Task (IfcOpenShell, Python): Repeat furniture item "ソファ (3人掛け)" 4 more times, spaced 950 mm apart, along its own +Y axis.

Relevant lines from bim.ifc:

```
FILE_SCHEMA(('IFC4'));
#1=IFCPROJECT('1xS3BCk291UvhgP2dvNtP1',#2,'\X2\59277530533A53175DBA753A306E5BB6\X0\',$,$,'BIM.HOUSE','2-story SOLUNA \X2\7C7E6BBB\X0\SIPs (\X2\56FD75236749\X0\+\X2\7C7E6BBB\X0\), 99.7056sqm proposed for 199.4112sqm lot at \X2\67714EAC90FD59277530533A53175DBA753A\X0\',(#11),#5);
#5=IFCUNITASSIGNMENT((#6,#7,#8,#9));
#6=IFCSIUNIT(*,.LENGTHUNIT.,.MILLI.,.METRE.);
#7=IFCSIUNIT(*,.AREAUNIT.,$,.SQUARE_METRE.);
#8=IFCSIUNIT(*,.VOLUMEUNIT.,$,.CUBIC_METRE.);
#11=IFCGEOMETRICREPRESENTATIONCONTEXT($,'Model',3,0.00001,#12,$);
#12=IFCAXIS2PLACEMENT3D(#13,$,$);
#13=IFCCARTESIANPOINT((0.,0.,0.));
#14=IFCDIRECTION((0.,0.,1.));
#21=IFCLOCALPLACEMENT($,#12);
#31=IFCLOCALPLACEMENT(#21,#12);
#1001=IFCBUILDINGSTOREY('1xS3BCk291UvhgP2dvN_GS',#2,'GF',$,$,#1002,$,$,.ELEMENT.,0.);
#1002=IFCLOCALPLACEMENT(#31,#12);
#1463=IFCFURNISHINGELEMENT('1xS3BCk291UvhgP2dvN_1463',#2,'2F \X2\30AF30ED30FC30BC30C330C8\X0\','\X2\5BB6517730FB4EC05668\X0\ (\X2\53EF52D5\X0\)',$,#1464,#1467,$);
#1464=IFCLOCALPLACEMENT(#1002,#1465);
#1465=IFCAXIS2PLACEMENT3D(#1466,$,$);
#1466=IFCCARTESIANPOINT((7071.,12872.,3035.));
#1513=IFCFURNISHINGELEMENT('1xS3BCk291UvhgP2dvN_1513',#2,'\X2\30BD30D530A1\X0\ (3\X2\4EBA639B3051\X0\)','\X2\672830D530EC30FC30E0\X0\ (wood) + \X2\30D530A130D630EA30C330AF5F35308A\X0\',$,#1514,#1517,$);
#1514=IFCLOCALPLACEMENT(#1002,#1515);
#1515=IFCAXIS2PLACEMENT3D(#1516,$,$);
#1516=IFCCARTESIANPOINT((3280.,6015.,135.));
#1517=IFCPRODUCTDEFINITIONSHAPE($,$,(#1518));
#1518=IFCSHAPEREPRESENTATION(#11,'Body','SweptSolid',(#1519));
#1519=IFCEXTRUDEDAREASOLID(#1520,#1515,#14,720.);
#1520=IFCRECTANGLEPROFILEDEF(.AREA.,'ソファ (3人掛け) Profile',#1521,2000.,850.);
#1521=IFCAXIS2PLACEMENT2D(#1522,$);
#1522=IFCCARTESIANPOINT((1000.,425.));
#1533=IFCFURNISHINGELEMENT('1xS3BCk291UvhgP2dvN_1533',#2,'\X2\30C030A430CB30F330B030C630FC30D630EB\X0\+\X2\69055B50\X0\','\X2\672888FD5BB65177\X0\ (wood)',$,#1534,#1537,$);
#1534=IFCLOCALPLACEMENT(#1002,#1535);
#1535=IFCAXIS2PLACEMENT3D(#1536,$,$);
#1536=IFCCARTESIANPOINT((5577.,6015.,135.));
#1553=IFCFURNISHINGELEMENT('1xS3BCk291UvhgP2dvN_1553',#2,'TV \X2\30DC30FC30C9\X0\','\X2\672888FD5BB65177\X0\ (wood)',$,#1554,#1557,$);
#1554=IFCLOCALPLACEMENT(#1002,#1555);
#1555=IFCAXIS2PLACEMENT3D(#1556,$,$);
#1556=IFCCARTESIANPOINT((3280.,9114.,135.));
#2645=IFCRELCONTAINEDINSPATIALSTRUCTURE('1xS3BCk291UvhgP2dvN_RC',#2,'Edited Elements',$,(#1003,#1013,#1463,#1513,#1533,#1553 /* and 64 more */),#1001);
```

```python
import ifcopenshell
import ifcopenshell.api.geometry
import ifcopenshell.api.root
import ifcopenshell.util.element
import ifcopenshell.util.placement
import ifcopenshell.util.unit

model = ifcopenshell.open("bim.ifc")
unit_scale = ifcopenshell.util.unit.calculate_unit_scale(model)


def reuse_history(source, copy):
    """copy_class also copies each property set's owner history, people and application; keep the originals."""
    for rel in copy.IsDefinedBy:
        if rel.is_a("IfcRelDefinesByProperties") and (history := rel.RelatingPropertyDefinition.OwnerHistory):
            rel.RelatingPropertyDefinition.OwnerHistory = source.OwnerHistory
            ifcopenshell.util.element.remove_deep2(model, history)


source = model.by_guid("1xS3BCk291UvhgP2dvN_1513")
base = ifcopenshell.util.placement.get_local_placement(source.ObjectPlacement)
step = base[:3, 1] * 0.95 / unit_scale

for i in range(1, 5):
    copy = ifcopenshell.api.root.copy_class(model, product=source)
    copy.Representation = ifcopenshell.util.element.copy_deep(
        model, source.Representation, exclude=["IfcGeometricRepresentationContext", "IfcRepresentationMap"]
    )
    reuse_history(source, copy)
    matrix = base.copy()
    matrix[:3, 3] += i * step
    print("added at", matrix[:3, 3].round(3) + 0.0)
    ifcopenshell.api.geometry.edit_object_placement(model, product=copy, matrix=matrix, is_si=False)

model.write("bim_rev.ifc")
```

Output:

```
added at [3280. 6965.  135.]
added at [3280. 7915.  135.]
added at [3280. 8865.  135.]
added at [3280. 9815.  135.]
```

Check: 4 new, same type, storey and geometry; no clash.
